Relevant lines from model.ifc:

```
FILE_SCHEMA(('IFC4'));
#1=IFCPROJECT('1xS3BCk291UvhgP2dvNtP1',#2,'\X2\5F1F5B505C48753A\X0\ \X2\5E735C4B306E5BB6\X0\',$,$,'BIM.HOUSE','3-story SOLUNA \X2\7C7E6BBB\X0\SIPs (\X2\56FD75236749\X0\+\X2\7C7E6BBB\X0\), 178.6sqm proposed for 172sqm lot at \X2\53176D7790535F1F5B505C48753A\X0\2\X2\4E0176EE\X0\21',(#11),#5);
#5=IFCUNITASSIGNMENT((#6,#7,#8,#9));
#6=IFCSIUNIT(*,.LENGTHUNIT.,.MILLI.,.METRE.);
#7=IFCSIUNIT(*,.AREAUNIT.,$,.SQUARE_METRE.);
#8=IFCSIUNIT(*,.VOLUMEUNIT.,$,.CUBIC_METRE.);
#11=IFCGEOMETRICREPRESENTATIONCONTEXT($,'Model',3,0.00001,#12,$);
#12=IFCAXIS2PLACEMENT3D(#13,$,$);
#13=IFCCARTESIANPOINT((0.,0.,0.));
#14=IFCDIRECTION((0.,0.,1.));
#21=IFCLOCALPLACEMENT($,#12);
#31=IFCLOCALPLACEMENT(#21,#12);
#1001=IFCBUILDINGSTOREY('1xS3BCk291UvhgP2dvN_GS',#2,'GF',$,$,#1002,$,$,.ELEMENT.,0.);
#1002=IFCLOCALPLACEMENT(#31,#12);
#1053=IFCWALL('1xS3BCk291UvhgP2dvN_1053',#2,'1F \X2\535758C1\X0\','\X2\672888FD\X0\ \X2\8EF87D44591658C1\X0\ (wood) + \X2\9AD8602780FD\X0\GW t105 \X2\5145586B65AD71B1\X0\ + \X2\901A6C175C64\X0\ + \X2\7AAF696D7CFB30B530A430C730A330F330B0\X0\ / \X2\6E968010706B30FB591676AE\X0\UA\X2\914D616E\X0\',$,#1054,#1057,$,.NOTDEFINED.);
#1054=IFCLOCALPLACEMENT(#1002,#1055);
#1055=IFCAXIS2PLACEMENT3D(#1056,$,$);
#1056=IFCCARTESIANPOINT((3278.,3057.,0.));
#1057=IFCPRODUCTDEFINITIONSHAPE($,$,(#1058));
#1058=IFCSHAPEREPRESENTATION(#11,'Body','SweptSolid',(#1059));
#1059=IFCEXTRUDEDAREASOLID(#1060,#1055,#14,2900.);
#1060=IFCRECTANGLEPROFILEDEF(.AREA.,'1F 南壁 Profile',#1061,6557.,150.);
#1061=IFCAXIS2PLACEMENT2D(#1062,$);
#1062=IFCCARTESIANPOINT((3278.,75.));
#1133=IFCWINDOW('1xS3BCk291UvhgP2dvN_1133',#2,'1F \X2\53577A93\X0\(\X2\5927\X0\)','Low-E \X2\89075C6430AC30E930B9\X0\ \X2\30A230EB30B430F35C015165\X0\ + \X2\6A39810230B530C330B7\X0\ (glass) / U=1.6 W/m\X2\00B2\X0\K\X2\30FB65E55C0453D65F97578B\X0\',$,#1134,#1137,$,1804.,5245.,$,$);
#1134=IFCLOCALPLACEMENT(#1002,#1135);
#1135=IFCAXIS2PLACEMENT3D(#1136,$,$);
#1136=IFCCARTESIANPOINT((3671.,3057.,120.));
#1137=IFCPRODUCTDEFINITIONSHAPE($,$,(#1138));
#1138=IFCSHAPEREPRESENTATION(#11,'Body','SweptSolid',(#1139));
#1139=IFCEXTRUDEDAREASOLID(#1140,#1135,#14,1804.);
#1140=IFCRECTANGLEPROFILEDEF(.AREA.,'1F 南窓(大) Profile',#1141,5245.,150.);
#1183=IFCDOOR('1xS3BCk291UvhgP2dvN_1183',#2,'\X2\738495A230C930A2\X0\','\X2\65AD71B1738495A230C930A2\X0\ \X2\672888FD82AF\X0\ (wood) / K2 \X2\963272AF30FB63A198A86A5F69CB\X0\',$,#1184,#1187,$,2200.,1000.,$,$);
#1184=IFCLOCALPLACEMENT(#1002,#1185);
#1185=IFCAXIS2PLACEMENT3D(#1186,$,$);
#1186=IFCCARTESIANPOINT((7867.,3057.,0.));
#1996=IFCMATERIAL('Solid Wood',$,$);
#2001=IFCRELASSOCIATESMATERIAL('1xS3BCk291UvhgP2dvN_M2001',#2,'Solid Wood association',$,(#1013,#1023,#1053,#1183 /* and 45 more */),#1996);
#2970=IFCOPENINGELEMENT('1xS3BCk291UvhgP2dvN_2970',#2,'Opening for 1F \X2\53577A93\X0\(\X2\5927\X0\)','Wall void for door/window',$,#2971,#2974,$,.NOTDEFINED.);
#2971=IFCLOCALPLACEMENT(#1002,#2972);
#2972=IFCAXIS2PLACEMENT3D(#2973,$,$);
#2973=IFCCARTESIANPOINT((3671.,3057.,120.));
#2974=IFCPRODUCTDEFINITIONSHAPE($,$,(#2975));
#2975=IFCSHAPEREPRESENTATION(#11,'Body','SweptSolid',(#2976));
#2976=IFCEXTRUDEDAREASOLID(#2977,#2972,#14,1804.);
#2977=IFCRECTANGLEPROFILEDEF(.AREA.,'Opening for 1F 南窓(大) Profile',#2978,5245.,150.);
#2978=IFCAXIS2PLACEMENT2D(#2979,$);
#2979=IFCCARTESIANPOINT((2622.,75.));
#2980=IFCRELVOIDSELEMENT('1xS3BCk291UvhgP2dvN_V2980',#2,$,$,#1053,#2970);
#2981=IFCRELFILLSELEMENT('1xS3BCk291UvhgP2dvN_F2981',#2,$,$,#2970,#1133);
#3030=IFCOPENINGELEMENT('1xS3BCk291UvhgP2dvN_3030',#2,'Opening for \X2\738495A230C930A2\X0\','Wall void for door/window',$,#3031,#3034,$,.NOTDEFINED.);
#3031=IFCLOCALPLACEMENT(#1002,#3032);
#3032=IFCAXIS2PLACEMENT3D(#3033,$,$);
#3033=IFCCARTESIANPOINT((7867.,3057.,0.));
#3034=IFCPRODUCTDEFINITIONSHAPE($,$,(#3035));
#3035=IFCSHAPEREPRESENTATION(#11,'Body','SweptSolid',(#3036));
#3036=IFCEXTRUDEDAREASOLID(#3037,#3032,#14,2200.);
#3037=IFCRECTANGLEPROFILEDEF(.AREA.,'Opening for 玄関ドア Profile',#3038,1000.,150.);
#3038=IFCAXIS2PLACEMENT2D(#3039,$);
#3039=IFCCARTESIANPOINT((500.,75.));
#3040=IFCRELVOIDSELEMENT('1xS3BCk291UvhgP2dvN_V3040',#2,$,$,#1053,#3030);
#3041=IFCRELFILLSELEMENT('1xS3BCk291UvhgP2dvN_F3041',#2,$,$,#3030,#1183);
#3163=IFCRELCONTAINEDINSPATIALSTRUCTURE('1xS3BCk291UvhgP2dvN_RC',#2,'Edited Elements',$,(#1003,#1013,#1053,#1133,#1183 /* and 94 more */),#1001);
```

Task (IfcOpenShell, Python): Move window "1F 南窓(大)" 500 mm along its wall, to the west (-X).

```python
import ifcopenshell
import ifcopenshell.api.geometry
import ifcopenshell.util.placement
import ifcopenshell.util.unit

model = ifcopenshell.open("model.ifc")
unit_scale = ifcopenshell.util.unit.calculate_unit_scale(model)

window = model.by_guid("1xS3BCk291UvhgP2dvN_1133")
opening = window.FillsVoids[0].RelatingOpeningElement
wall = opening.VoidsElements[0].RelatingBuildingElement

wall_matrix = ifcopenshell.util.placement.get_local_placement(wall.ObjectPlacement)
shift = wall_matrix[:3, 0] * -0.5 / unit_scale
before = ifcopenshell.util.placement.get_local_placement(window.ObjectPlacement)[:3, 3].copy()

# The window is not placed relative to its opening, so move both.
for product in (opening, window):
    matrix = ifcopenshell.util.placement.get_local_placement(product.ObjectPlacement)
    matrix[:3, 3] += shift
    ifcopenshell.api.geometry.edit_object_placement(model, product=product, matrix=matrix, is_si=False)

after = ifcopenshell.util.placement.get_local_placement(window.ObjectPlacement)[:3, 3]
print("window moved by", (after - before).round(3) + 0.0)

model.write("model_v2.ifc")
```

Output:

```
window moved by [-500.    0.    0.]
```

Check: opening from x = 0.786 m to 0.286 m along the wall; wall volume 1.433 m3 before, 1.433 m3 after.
